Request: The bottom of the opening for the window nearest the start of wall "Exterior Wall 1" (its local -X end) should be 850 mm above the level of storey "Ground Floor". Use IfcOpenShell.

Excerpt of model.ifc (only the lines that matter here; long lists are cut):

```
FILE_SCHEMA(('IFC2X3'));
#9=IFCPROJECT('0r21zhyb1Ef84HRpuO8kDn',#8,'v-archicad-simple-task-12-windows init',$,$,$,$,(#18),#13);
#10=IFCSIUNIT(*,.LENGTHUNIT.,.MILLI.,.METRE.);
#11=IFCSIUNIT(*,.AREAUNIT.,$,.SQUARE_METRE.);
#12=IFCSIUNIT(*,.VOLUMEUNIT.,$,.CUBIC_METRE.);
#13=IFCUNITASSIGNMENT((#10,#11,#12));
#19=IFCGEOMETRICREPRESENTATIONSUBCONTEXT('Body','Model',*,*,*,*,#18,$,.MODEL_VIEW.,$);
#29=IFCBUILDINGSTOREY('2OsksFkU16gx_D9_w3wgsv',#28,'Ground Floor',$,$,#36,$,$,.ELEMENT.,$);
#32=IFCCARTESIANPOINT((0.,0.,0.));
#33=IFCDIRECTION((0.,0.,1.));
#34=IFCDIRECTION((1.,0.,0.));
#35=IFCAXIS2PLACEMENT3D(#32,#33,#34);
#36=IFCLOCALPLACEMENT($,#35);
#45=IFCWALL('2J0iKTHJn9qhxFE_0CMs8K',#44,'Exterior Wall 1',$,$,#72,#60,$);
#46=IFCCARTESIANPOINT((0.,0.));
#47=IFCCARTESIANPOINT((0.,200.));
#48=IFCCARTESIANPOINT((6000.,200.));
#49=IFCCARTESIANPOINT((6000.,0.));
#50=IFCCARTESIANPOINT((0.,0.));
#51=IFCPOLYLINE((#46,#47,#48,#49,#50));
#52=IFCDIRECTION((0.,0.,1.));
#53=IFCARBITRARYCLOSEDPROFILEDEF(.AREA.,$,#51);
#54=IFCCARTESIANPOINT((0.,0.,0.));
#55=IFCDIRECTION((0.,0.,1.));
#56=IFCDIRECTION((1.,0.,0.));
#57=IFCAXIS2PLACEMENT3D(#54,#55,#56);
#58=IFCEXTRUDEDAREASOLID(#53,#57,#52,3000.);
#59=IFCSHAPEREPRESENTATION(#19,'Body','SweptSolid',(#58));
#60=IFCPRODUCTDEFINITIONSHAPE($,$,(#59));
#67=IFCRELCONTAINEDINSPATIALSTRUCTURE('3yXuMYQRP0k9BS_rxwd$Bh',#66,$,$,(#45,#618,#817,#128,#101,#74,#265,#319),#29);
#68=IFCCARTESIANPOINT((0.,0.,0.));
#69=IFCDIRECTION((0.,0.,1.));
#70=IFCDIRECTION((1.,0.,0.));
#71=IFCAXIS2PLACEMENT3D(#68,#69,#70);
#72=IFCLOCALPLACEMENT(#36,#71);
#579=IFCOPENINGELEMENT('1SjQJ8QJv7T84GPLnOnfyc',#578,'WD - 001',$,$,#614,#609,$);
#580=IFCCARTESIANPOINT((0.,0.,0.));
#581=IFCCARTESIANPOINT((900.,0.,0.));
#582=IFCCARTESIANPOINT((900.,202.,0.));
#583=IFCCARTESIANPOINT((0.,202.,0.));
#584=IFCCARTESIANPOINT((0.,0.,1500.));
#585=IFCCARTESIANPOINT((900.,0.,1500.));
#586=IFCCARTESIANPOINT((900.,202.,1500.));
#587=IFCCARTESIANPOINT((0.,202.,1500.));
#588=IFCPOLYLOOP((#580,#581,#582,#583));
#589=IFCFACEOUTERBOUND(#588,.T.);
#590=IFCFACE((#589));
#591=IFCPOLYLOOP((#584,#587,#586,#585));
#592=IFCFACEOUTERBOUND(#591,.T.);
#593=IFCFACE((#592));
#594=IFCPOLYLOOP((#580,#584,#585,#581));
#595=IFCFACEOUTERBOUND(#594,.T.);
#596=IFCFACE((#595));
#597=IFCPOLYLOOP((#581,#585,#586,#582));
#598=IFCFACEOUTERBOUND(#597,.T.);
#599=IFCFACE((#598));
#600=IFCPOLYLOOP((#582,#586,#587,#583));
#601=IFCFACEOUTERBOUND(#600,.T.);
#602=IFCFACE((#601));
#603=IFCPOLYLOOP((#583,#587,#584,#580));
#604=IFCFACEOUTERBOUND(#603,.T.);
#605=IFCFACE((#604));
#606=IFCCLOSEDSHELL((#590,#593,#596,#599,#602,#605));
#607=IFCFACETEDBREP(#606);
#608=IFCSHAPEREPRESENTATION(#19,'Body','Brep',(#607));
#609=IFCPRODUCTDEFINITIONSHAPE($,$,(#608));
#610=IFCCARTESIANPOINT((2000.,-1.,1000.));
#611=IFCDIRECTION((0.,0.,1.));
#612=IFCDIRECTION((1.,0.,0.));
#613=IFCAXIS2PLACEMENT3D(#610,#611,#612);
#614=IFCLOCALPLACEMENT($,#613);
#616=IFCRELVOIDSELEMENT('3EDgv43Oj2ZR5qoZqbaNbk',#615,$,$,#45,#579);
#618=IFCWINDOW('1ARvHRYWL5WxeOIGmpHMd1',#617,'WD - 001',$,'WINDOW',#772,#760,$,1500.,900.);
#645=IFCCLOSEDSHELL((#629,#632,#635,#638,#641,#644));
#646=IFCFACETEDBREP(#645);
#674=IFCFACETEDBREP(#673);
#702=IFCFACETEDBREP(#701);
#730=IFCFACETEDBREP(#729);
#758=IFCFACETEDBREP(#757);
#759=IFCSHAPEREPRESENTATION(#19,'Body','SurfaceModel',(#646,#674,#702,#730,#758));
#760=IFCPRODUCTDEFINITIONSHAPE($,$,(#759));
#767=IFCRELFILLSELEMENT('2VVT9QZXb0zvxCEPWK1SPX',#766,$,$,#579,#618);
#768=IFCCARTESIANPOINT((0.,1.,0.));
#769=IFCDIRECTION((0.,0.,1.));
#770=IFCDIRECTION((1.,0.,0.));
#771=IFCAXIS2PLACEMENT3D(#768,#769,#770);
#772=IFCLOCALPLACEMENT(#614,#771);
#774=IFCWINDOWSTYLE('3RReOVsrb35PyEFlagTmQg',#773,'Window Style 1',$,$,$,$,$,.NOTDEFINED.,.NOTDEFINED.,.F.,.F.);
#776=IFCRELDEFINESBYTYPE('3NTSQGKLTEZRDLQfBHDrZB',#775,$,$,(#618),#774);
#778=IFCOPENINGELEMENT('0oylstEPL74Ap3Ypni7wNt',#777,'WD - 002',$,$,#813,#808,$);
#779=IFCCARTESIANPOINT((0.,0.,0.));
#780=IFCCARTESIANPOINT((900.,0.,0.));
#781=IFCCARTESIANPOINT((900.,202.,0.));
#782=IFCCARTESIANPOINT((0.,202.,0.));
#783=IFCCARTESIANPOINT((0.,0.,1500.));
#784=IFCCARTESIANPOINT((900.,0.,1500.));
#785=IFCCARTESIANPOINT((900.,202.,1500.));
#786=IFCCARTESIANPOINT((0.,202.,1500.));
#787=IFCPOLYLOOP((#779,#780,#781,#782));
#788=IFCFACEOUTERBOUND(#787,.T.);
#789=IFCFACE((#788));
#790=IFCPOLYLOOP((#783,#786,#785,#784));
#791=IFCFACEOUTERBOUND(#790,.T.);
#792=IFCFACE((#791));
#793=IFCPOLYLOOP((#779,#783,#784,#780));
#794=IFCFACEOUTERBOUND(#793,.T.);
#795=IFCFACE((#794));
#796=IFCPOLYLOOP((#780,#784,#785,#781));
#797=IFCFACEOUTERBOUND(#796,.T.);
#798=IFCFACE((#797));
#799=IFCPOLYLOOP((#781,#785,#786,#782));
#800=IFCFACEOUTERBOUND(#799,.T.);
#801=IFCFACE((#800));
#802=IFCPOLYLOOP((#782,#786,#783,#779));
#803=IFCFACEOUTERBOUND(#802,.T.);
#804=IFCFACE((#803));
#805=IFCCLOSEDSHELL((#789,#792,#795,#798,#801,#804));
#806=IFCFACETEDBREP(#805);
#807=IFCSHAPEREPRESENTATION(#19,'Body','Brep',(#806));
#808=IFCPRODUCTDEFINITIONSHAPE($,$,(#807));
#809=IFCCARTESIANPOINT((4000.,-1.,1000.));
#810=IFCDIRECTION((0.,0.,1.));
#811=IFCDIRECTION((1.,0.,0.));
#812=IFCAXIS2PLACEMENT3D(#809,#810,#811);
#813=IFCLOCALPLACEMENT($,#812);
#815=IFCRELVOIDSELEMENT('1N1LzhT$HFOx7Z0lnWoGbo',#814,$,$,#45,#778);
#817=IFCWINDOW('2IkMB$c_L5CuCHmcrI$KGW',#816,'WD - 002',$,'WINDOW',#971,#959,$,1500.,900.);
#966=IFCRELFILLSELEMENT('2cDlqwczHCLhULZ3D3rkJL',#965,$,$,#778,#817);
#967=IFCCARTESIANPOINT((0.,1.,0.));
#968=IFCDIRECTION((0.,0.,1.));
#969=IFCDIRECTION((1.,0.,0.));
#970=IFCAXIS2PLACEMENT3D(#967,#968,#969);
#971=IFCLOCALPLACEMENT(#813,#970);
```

```python
import numpy as np
import ifcopenshell
import ifcopenshell.api.geometry
import ifcopenshell.geom
import ifcopenshell.util.element
import ifcopenshell.util.placement
import ifcopenshell.util.shape
import ifcopenshell.util.unit

model = ifcopenshell.open("model.ifc")
unit_scale = ifcopenshell.util.unit.calculate_unit_scale(model)

window = model.by_guid("1ARvHRYWL5WxeOIGmpHMd1")
opening = window.FillsVoids[0].RelatingOpeningElement
storey = ifcopenshell.util.element.get_container(window, ifc_class="IfcBuildingStorey")
level = ifcopenshell.util.placement.get_local_placement(storey.ObjectPlacement)[2, 3]

# The opening's origin need not be at the sill, so measure its lowest point.
shape = ifcopenshell.geom.create_shape(ifcopenshell.geom.settings(), opening)
bottom = ifcopenshell.util.shape.get_shape_bottom_elevation(shape, shape.geometry) / unit_scale
dz = level + 0.85 / unit_scale - bottom

shift = np.array([0.0, 0.0, dz])
# The window is placed relative to its opening, so it follows when the opening moves.
matrix = ifcopenshell.util.placement.get_local_placement(opening.ObjectPlacement)
matrix[:3, 3] += shift
ifcopenshell.api.geometry.edit_object_placement(
    model, product=opening, matrix=matrix, is_si=False, should_transform_children=True
)

print(f"moved by {dz * unit_scale:+.3f} m")

model.write("model-out.ifc")
```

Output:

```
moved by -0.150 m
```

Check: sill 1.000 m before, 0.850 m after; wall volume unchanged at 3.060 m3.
